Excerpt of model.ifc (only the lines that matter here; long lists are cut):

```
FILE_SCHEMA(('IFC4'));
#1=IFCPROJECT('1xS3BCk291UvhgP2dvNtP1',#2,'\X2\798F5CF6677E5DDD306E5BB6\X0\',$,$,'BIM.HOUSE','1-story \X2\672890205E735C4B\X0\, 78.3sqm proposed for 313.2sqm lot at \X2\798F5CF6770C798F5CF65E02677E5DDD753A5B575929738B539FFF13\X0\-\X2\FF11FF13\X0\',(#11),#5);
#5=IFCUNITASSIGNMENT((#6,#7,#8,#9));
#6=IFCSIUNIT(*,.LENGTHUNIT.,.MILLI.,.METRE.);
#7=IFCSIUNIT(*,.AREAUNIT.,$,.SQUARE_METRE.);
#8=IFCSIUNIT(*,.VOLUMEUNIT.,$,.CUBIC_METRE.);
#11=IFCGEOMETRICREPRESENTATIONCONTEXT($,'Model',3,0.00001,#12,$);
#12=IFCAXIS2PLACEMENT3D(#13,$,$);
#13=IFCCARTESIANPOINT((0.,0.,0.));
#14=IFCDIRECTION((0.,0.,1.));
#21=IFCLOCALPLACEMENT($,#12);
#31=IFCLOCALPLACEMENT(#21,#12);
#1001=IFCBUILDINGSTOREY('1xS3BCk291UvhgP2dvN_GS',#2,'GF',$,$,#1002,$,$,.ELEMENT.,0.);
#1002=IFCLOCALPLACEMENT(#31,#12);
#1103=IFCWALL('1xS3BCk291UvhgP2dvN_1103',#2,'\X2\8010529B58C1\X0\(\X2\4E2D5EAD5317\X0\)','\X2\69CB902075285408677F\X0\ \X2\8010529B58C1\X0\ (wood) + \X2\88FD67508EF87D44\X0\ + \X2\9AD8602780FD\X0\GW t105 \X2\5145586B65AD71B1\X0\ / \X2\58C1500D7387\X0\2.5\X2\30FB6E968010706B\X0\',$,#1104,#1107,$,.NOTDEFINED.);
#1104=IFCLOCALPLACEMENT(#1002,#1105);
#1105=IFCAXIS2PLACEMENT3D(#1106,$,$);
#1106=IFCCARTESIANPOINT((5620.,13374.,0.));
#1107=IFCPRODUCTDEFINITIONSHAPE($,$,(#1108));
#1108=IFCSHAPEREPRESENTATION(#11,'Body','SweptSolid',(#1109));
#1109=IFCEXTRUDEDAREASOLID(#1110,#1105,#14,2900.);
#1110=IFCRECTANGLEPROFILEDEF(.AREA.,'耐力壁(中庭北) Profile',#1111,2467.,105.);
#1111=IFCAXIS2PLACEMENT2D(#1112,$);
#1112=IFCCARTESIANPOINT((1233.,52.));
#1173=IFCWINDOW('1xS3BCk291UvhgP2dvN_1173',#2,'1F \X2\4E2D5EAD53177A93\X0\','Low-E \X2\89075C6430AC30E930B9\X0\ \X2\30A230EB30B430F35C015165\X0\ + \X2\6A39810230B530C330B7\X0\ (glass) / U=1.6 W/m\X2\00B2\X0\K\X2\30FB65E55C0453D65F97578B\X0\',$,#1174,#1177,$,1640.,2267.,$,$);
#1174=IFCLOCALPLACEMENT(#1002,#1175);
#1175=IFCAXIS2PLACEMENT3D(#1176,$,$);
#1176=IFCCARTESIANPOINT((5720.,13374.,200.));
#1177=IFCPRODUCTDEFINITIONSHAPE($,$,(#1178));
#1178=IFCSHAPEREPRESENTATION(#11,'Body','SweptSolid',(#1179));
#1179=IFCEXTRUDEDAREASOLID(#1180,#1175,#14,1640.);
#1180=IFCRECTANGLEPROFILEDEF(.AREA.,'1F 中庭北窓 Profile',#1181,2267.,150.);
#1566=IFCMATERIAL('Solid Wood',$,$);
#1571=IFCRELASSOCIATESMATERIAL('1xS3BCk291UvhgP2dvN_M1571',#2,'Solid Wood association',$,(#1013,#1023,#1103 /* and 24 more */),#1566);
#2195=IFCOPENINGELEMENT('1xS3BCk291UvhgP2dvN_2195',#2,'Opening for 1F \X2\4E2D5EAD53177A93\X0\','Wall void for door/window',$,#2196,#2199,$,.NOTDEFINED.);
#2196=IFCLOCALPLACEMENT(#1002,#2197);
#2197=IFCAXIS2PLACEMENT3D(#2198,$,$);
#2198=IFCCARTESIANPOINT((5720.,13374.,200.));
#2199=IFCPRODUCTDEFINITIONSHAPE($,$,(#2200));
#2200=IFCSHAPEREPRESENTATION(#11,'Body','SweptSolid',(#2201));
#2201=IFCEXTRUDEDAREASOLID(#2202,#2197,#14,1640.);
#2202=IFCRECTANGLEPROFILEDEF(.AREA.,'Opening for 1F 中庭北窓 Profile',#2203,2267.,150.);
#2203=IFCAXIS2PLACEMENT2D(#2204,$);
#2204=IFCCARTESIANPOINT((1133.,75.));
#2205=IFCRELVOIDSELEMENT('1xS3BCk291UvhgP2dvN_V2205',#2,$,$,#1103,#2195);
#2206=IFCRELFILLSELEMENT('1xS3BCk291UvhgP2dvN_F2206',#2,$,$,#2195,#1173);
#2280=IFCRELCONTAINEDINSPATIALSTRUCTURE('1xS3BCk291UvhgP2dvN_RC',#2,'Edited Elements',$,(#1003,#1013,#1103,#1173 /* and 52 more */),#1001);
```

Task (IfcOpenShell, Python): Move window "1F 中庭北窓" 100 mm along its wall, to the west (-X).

```python
import ifcopenshell
import ifcopenshell.api.geometry
import ifcopenshell.util.placement
import ifcopenshell.util.unit

model = ifcopenshell.open("model.ifc")
unit_scale = ifcopenshell.util.unit.calculate_unit_scale(model)

window = model.by_guid("1xS3BCk291UvhgP2dvN_1173")
opening = window.FillsVoids[0].RelatingOpeningElement
wall = opening.VoidsElements[0].RelatingBuildingElement

wall_matrix = ifcopenshell.util.placement.get_local_placement(wall.ObjectPlacement)
shift = wall_matrix[:3, 0] * -0.1 / unit_scale
before = ifcopenshell.util.placement.get_local_placement(window.ObjectPlacement)[:3, 3].copy()

# The window is not placed relative to its opening, so move both.
for product in (opening, window):
    matrix = ifcopenshell.util.placement.get_local_placement(product.ObjectPlacement)
    matrix[:3, 3] += shift
    ifcopenshell.api.geometry.edit_object_placement(model, product=product, matrix=matrix, is_si=False)

after = ifcopenshell.util.placement.get_local_placement(window.ObjectPlacement)[:3, 3]
print("window moved by", (after - before).round(3) + 0.0)

model.write("model_edited.ifc")
```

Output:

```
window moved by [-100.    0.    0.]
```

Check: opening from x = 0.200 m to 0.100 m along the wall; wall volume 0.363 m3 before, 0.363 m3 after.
